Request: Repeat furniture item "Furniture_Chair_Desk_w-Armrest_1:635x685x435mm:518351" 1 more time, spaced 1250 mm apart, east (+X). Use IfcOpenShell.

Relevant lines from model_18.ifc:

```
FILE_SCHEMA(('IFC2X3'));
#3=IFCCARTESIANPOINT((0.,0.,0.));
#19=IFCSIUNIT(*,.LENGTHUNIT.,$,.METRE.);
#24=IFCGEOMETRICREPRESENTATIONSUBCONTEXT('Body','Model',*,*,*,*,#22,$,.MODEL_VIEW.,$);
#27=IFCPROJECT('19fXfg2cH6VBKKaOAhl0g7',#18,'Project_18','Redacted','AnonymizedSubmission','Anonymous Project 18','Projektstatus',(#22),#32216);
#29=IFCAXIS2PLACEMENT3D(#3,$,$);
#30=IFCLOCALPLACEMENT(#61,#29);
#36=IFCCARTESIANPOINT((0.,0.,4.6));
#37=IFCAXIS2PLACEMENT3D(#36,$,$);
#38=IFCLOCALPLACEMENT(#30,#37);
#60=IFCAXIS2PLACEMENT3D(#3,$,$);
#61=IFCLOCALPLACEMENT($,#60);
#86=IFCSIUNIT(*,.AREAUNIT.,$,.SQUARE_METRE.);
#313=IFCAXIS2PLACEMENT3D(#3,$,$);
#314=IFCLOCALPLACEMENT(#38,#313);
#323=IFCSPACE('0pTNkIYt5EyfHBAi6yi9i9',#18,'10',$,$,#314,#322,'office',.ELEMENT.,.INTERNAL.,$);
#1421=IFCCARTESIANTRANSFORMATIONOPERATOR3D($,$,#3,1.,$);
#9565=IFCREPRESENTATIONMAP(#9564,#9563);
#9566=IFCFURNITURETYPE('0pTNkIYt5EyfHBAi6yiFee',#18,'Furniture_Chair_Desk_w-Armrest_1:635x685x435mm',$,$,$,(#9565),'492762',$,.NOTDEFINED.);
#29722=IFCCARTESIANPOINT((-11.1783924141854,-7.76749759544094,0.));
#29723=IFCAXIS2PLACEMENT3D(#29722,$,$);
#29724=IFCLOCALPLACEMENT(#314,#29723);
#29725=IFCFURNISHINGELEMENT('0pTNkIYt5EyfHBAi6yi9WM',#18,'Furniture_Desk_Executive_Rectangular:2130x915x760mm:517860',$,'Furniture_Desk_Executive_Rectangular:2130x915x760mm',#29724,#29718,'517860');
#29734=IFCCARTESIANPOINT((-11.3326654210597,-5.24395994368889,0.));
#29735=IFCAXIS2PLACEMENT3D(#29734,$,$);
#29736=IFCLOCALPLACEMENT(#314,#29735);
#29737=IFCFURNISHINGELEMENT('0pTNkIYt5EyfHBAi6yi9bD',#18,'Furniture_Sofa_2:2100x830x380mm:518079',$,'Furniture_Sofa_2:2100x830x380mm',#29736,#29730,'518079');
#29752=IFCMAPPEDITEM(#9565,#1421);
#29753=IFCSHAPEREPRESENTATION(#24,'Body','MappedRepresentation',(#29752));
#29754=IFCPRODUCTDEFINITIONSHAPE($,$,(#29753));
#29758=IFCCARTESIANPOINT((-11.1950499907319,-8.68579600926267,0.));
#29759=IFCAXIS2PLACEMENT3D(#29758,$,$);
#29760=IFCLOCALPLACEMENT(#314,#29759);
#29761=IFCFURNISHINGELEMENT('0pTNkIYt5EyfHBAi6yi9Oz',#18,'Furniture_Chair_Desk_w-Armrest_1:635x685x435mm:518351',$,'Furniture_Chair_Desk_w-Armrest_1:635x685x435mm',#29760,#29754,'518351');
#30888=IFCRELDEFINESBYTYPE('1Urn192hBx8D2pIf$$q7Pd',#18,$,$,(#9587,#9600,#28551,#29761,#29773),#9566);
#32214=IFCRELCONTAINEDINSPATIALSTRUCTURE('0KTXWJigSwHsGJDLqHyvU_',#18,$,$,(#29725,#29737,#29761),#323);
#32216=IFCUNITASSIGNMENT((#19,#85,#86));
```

```python
import numpy as np
import ifcopenshell
import ifcopenshell.api.geometry
import ifcopenshell.api.root
import ifcopenshell.util.element
import ifcopenshell.util.placement

model = ifcopenshell.open("model_18.ifc")


def reuse_history(source, copy):
    """copy_class also copies each property set's owner history, people and application; keep the originals."""
    for rel in copy.IsDefinedBy:
        if rel.is_a("IfcRelDefinesByProperties") and (history := rel.RelatingPropertyDefinition.OwnerHistory):
            rel.RelatingPropertyDefinition.OwnerHistory = source.OwnerHistory
            ifcopenshell.util.element.remove_deep2(model, history)


source = model.by_id(29761)
base = ifcopenshell.util.placement.get_local_placement(source.ObjectPlacement)
step = np.array([1.0, 0.0, 0.0]) * 1.25

for i in range(1, 2):
    copy = ifcopenshell.api.root.copy_class(model, product=source)
    copy.Representation = ifcopenshell.util.element.copy_deep(
        model, source.Representation, exclude=["IfcGeometricRepresentationContext", "IfcRepresentationMap"]
    )
    copy.Name = "Furniture_Chair_Desk_w-Armrest_1:635x685x435mm"
    copy.Tag = None
    reuse_history(source, copy)
    matrix = base.copy()
    matrix[:3, 3] += i * step
    print("added at", matrix[:3, 3].round(3) + 0.0)
    ifcopenshell.api.geometry.edit_object_placement(model, product=copy, matrix=matrix, is_si=False)

model.write("model_18_edited.ifc")
```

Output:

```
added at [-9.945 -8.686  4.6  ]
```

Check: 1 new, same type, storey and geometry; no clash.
